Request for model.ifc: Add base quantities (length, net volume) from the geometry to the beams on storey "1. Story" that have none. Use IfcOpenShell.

First a look at what the model holds.

```python
import ifcopenshell
import ifcopenshell.util.element
import ifcopenshell.util.unit

model = ifcopenshell.open("model.ifc")
print(model.schema)
for unit_type in ("LENGTHUNIT", "AREAUNIT", "VOLUMEUNIT"):
    print(unit_type, ifcopenshell.util.unit.calculate_unit_scale(model, unit_type))
storey = next(s for s in model.by_type("IfcBuildingStorey") if s.Name == "1. Story")
beams = [e for e in ifcopenshell.util.element.get_decomposition(storey) if e.is_a("IfcBeam")]
for e in sorted(beams, key=lambda e: e.id()):
    print(e.id(), e.is_a(), e.Name, list(ifcopenshell.util.element.get_psets(e, qtos_only=True)), sep=" | ")
```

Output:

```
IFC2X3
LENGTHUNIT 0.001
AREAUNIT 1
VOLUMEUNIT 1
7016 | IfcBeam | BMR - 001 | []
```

```python
import ifcopenshell
import ifcopenshell.api.pset
import ifcopenshell.geom
import ifcopenshell.util.element
import ifcopenshell.util.shape
import ifcopenshell.util.unit

model = ifcopenshell.open("model.ifc")
unit_scale = ifcopenshell.util.unit.calculate_unit_scale(model)
volume_scale = ifcopenshell.util.unit.calculate_unit_scale(model, "VOLUMEUNIT")
settings = ifcopenshell.geom.settings()

storey = next(s for s in model.by_type("IfcBuildingStorey") if s.Name == "1. Story")
beams = [e for e in ifcopenshell.util.element.get_decomposition(storey) if e.is_a("IfcBeam")]

for e in sorted(beams, key=lambda e: e.id()):
    if ifcopenshell.util.element.get_psets(e, qtos_only=True, should_inherit=False):
        continue
    # Geometry comes back in metres, in the element's own axes.
    shape = ifcopenshell.geom.create_shape(settings, e)
    values = {
        "Length": ifcopenshell.util.shape.get_max_xyz(shape.geometry) / unit_scale,
        "NetVolume": ifcopenshell.util.shape.get_volume(shape.geometry) / volume_scale,
    }
    qto = ifcopenshell.api.pset.add_qto(model, product=e, name="BaseQuantities")
    ifcopenshell.api.pset.edit_qto(model, qto=qto, properties=values)
    print(e.id(), {k: round(v, 3) for k, v in values.items()})

model.write("model-out.ifc")
```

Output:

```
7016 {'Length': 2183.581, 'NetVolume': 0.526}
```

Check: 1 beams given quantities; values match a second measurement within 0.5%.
